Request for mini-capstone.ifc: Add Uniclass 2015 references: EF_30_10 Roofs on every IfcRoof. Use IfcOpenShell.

First a look at what the model holds.

```python
import ifcopenshell

model = ifcopenshell.open("mini-capstone.ifc")
print(model.schema)
print("classifications:", [c.Name for c in model.by_type("IfcClassification")])
for ifc_class in ("IfcDoor", "IfcRoof", "IfcStair", "IfcWall", "IfcWindow"):
    print(ifc_class, len(model.by_type(ifc_class)))
```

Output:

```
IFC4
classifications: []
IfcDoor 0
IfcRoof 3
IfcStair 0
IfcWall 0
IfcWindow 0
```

```python
import ifcopenshell
import ifcopenshell.api.classification

model = ifcopenshell.open("mini-capstone.ifc")

system = ifcopenshell.api.classification.add_classification(model, classification="Uniclass 2015")

codes = {
    "IfcRoof": ("EF_30_10", "Roofs"),
}
for ifc_class, (code, name) in codes.items():
    products = model.by_type(ifc_class)
    ifcopenshell.api.classification.add_reference(
        model, products=products, classification=system, identification=code, name=name
    )
    print(code, len(products))

model.write("mini-capstone_updated.ifc")
```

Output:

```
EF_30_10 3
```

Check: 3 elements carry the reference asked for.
